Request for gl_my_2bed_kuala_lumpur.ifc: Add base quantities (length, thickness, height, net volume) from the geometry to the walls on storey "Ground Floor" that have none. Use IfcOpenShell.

First a look at what the model holds.

```python
import ifcopenshell
import ifcopenshell.util.element
import ifcopenshell.util.unit

model = ifcopenshell.open("gl_my_2bed_kuala_lumpur.ifc")
print(model.schema)
for unit_type in ("LENGTHUNIT", "AREAUNIT", "VOLUMEUNIT"):
    print(unit_type, ifcopenshell.util.unit.calculate_unit_scale(model, unit_type))
storey = next(s for s in model.by_type("IfcBuildingStorey") if s.Name == "Ground Floor")
walls = [e for e in ifcopenshell.util.element.get_decomposition(storey) if e.is_a("IfcWall")]
for e in sorted(walls, key=lambda e: e.id()):
    print(e.id(), e.is_a(), e.Name, list(ifcopenshell.util.element.get_psets(e, qtos_only=True)), sep=" | ")
```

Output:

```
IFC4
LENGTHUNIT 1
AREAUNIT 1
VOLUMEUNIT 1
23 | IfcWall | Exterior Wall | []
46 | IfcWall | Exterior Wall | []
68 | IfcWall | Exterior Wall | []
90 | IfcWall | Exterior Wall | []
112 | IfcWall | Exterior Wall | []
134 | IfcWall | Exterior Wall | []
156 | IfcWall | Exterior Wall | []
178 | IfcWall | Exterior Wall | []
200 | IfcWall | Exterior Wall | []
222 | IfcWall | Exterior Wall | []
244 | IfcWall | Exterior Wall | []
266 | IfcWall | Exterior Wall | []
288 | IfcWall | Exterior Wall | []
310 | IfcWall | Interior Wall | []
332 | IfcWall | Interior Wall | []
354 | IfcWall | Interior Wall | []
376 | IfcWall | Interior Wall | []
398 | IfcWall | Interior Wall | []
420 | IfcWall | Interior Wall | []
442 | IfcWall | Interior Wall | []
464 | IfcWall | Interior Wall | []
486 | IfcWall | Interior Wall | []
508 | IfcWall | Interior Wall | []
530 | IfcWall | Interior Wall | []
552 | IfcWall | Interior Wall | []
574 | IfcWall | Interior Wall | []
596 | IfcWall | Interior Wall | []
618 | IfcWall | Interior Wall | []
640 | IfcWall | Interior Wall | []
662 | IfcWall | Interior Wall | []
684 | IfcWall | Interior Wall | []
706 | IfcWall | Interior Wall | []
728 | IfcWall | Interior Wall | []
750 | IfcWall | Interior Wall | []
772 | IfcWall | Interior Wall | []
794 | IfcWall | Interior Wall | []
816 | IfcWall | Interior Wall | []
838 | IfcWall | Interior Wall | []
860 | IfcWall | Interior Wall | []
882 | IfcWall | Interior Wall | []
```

```python
import ifcopenshell
import ifcopenshell.api.pset
import ifcopenshell.geom
import ifcopenshell.util.element
import ifcopenshell.util.shape
import ifcopenshell.util.unit

model = ifcopenshell.open("gl_my_2bed_kuala_lumpur.ifc")
unit_scale = ifcopenshell.util.unit.calculate_unit_scale(model)
volume_scale = ifcopenshell.util.unit.calculate_unit_scale(model, "VOLUMEUNIT")
settings = ifcopenshell.geom.settings()

storey = next(s for s in model.by_type("IfcBuildingStorey") if s.Name == "Ground Floor")
walls = [e for e in ifcopenshell.util.element.get_decomposition(storey) if e.is_a("IfcWall")]

for e in sorted(walls, key=lambda e: e.id()):
    if ifcopenshell.util.element.get_psets(e, qtos_only=True, should_inherit=False):
        continue
    # Geometry comes back in metres, in the element's own axes.
    shape = ifcopenshell.geom.create_shape(settings, e)
    values = {
        "Length": ifcopenshell.util.shape.get_x(shape.geometry) / unit_scale,
        "Width": ifcopenshell.util.shape.get_y(shape.geometry) / unit_scale,
        "Height": ifcopenshell.util.shape.get_z(shape.geometry) / unit_scale,
        "NetVolume": ifcopenshell.util.shape.get_volume(shape.geometry) / volume_scale,
    }
    qto = ifcopenshell.api.pset.add_qto(model, product=e, name="Qto_WallBaseQuantities")
    ifcopenshell.api.pset.edit_qto(model, qto=qto, properties=values)
    print(e.id(), {k: round(v, 3) for k, v in values.items()})

model.write("gl_my_2bed_kuala_lumpur_updated.ifc")
```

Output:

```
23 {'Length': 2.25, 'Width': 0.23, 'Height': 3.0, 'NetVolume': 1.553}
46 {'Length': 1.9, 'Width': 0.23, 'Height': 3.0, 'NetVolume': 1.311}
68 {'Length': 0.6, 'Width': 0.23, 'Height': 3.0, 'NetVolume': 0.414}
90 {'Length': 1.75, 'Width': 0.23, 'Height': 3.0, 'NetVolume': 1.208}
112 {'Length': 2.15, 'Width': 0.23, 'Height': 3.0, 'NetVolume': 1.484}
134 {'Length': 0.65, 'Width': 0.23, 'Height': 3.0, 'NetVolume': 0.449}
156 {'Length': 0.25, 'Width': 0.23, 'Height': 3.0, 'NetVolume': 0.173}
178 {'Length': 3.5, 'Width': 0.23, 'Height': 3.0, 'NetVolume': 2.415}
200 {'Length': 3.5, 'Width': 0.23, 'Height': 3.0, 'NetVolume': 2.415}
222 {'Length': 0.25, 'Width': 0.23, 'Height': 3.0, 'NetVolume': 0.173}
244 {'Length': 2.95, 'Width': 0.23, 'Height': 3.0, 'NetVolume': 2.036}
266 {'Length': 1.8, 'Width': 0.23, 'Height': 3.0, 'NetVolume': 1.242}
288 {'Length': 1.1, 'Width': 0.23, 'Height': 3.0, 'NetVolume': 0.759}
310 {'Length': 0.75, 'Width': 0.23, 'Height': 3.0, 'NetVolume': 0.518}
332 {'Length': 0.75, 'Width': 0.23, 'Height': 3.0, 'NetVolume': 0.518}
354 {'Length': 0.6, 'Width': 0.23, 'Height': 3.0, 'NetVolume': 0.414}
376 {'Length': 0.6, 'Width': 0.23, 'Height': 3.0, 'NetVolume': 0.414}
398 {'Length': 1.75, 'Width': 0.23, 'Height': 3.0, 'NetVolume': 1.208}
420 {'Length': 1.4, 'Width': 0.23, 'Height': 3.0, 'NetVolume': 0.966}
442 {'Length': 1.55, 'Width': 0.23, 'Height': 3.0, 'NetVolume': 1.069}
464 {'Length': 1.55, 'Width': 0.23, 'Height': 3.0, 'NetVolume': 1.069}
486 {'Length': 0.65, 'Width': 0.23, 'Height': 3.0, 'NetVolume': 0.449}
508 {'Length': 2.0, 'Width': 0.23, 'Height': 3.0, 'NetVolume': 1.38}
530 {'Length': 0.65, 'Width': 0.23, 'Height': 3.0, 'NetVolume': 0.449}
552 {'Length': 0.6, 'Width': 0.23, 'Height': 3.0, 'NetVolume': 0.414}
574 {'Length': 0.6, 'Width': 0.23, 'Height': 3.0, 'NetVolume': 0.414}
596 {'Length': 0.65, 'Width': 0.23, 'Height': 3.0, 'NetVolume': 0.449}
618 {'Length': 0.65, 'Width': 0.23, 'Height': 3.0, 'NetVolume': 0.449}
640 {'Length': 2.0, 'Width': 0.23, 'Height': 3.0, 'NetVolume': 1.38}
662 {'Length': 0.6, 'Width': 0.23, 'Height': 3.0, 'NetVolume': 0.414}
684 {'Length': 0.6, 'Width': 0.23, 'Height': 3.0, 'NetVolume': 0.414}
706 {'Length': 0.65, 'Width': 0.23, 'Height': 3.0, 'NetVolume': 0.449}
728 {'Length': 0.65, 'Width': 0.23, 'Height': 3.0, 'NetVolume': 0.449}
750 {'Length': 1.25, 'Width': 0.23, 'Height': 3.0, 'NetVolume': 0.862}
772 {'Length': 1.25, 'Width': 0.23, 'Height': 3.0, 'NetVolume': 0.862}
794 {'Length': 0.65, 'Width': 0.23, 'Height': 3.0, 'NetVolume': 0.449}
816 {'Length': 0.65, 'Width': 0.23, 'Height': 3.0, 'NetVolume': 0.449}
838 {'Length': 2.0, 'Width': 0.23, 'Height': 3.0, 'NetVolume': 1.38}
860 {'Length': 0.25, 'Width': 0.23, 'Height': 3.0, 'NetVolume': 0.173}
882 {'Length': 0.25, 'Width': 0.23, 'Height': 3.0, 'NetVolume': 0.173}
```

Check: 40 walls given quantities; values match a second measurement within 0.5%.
